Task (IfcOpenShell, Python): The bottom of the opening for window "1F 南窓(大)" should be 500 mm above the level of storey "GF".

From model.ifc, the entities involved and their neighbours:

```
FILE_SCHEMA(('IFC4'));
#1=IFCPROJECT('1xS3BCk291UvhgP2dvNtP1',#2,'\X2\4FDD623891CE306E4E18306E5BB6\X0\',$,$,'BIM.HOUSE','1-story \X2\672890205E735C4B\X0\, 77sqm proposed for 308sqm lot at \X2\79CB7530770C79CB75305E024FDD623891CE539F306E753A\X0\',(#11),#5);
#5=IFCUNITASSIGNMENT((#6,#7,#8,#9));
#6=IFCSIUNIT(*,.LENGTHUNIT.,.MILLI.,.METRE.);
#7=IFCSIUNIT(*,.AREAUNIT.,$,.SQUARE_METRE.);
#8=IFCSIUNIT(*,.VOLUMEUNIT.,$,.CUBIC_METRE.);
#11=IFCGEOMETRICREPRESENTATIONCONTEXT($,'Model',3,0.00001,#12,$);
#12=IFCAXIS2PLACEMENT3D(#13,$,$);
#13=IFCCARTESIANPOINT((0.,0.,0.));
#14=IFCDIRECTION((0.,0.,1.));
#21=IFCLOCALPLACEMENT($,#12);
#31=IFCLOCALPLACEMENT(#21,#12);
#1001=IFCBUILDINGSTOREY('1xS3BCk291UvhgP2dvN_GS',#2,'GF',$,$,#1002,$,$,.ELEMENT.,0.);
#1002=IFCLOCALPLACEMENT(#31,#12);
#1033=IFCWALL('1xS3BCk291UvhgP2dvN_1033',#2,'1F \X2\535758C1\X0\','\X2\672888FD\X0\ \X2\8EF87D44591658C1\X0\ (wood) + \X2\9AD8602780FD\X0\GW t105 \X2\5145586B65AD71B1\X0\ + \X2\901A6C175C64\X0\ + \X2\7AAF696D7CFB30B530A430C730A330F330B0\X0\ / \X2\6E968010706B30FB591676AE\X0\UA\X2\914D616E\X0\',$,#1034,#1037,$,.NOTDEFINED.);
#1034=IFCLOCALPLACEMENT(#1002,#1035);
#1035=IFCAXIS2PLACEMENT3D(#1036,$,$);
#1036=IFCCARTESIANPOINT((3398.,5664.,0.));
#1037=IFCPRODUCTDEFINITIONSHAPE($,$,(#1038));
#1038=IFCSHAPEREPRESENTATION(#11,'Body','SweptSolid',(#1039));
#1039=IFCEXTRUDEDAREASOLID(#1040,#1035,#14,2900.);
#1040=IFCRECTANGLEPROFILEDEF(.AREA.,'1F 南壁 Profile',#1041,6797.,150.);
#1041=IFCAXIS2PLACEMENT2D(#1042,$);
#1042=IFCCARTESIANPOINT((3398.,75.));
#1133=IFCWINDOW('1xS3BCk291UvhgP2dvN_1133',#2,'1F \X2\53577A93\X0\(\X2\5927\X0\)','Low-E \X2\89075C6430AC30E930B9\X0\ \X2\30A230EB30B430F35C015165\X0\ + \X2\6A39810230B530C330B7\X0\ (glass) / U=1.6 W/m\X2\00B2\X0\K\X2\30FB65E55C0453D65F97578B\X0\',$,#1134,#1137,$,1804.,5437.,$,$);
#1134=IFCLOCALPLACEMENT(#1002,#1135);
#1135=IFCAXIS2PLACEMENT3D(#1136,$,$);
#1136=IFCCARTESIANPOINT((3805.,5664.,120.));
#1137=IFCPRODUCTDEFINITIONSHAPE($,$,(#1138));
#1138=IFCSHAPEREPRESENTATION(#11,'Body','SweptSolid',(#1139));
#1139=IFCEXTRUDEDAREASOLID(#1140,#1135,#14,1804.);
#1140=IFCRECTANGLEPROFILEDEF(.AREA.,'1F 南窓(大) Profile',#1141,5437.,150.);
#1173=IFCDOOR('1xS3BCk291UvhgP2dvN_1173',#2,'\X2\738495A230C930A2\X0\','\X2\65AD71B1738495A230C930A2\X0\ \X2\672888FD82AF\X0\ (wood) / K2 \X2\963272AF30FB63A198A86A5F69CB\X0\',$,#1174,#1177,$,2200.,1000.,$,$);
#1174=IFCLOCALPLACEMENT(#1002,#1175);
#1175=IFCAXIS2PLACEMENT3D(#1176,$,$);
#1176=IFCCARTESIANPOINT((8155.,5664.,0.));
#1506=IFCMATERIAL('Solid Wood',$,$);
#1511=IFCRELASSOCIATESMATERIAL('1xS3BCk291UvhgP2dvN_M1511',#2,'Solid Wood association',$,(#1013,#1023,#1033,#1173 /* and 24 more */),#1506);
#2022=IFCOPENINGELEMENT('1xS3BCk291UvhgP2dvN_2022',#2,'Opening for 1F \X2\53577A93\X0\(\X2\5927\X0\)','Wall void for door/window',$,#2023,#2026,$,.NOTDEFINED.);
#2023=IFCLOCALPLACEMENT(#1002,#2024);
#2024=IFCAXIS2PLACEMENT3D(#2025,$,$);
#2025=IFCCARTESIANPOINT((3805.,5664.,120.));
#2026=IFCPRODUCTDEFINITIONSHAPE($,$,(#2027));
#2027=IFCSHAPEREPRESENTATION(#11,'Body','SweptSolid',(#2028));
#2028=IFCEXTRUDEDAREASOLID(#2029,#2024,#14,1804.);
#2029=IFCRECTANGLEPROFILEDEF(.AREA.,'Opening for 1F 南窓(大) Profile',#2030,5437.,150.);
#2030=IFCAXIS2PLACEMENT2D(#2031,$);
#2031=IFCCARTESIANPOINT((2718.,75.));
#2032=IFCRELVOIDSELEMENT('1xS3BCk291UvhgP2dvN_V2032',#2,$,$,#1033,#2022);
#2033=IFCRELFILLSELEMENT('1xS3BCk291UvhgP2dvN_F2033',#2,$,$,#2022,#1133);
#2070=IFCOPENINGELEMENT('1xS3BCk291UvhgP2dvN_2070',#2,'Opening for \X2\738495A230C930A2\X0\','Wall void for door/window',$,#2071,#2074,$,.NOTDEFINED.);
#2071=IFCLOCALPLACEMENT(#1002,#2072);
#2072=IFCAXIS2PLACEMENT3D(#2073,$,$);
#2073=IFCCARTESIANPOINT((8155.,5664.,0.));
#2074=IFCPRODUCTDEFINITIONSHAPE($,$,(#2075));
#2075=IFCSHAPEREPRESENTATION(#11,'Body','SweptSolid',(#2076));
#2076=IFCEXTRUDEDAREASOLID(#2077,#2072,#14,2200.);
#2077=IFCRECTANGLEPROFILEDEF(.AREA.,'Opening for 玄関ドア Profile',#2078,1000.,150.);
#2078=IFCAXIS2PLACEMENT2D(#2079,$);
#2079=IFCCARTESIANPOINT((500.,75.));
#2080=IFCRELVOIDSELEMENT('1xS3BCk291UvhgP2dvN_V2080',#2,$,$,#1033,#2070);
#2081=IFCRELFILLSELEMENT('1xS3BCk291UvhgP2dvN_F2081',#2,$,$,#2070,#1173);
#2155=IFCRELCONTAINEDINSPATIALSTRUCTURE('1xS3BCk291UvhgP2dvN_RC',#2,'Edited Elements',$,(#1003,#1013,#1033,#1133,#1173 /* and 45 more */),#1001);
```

```python
import numpy as np
import ifcopenshell
import ifcopenshell.api.geometry
import ifcopenshell.geom
import ifcopenshell.util.element
import ifcopenshell.util.placement
import ifcopenshell.util.shape
import ifcopenshell.util.unit

model = ifcopenshell.open("model.ifc")
unit_scale = ifcopenshell.util.unit.calculate_unit_scale(model)

window = model.by_guid("1xS3BCk291UvhgP2dvN_1133")
opening = window.FillsVoids[0].RelatingOpeningElement
storey = ifcopenshell.util.element.get_container(window, ifc_class="IfcBuildingStorey")
level = ifcopenshell.util.placement.get_local_placement(storey.ObjectPlacement)[2, 3]

# The opening's origin need not be at the sill, so measure its lowest point.
shape = ifcopenshell.geom.create_shape(ifcopenshell.geom.settings(), opening)
bottom = ifcopenshell.util.shape.get_shape_bottom_elevation(shape, shape.geometry) / unit_scale
dz = level + 500.0 - bottom

shift = np.array([0.0, 0.0, dz])
# The window is not placed relative to its opening, so move both.
for product in (opening, window):
    matrix = ifcopenshell.util.placement.get_local_placement(product.ObjectPlacement)
    matrix[:3, 3] += shift
    ifcopenshell.api.geometry.edit_object_placement(model, product=product, matrix=matrix, is_si=False)

print(f"moved by {dz * unit_scale:+.3f} m")

model.write("model_v2.ifc")
```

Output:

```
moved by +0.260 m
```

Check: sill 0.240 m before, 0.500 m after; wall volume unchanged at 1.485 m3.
